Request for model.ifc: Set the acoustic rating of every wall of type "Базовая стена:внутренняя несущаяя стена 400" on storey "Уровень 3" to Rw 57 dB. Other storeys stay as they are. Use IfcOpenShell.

First a look at what the model holds.

```python
import ifcopenshell
import ifcopenshell.util.element

model = ifcopenshell.open("model.ifc")
print(model.schema)
storey = next(s for s in model.by_type("IfcBuildingStorey") if s.Name == "Уровень 3")
walls = [e for e in ifcopenshell.util.element.get_decomposition(storey) if e.is_a("IfcWall")]
seen = {}
for e in walls:
    element_type = ifcopenshell.util.element.get_type(e)
    key = (element_type.Name if element_type != e and element_type else None, ifcopenshell.util.element.get_pset(e, "Pset_WallCommon", "AcousticRating"))
    seen[key] = seen.get(key, 0) + 1
for (name, value), count in sorted(seen.items(), key=str):
    print(count, "x", name, "|", value)
```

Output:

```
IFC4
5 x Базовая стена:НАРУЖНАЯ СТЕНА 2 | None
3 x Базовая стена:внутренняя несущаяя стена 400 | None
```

```python
import ifcopenshell
import ifcopenshell.api.pset
import ifcopenshell.util.element

model = ifcopenshell.open("model.ifc")

storey = next(s for s in model.by_type("IfcBuildingStorey") if s.Name == "Уровень 3")
walls = [e for e in ifcopenshell.util.element.get_decomposition(storey) if e.is_a("IfcWall")]

count = 0
for e in walls:
    element_type = ifcopenshell.util.element.get_type(e)
    if element_type in (None, e) or element_type.Name != "Базовая стена:внутренняя несущаяя стена 400":
        continue
    # add_pset returns the element's existing set when there is one.
    pset = ifcopenshell.api.pset.add_pset(model, product=e, name="Pset_WallCommon")
    ifcopenshell.api.pset.edit_pset(model, pset=pset, properties={"AcousticRating": "Rw 57 dB"})
    count += 1

print(count, "walls updated")

model.write("model-out.ifc")
```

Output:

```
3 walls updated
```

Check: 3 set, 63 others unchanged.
